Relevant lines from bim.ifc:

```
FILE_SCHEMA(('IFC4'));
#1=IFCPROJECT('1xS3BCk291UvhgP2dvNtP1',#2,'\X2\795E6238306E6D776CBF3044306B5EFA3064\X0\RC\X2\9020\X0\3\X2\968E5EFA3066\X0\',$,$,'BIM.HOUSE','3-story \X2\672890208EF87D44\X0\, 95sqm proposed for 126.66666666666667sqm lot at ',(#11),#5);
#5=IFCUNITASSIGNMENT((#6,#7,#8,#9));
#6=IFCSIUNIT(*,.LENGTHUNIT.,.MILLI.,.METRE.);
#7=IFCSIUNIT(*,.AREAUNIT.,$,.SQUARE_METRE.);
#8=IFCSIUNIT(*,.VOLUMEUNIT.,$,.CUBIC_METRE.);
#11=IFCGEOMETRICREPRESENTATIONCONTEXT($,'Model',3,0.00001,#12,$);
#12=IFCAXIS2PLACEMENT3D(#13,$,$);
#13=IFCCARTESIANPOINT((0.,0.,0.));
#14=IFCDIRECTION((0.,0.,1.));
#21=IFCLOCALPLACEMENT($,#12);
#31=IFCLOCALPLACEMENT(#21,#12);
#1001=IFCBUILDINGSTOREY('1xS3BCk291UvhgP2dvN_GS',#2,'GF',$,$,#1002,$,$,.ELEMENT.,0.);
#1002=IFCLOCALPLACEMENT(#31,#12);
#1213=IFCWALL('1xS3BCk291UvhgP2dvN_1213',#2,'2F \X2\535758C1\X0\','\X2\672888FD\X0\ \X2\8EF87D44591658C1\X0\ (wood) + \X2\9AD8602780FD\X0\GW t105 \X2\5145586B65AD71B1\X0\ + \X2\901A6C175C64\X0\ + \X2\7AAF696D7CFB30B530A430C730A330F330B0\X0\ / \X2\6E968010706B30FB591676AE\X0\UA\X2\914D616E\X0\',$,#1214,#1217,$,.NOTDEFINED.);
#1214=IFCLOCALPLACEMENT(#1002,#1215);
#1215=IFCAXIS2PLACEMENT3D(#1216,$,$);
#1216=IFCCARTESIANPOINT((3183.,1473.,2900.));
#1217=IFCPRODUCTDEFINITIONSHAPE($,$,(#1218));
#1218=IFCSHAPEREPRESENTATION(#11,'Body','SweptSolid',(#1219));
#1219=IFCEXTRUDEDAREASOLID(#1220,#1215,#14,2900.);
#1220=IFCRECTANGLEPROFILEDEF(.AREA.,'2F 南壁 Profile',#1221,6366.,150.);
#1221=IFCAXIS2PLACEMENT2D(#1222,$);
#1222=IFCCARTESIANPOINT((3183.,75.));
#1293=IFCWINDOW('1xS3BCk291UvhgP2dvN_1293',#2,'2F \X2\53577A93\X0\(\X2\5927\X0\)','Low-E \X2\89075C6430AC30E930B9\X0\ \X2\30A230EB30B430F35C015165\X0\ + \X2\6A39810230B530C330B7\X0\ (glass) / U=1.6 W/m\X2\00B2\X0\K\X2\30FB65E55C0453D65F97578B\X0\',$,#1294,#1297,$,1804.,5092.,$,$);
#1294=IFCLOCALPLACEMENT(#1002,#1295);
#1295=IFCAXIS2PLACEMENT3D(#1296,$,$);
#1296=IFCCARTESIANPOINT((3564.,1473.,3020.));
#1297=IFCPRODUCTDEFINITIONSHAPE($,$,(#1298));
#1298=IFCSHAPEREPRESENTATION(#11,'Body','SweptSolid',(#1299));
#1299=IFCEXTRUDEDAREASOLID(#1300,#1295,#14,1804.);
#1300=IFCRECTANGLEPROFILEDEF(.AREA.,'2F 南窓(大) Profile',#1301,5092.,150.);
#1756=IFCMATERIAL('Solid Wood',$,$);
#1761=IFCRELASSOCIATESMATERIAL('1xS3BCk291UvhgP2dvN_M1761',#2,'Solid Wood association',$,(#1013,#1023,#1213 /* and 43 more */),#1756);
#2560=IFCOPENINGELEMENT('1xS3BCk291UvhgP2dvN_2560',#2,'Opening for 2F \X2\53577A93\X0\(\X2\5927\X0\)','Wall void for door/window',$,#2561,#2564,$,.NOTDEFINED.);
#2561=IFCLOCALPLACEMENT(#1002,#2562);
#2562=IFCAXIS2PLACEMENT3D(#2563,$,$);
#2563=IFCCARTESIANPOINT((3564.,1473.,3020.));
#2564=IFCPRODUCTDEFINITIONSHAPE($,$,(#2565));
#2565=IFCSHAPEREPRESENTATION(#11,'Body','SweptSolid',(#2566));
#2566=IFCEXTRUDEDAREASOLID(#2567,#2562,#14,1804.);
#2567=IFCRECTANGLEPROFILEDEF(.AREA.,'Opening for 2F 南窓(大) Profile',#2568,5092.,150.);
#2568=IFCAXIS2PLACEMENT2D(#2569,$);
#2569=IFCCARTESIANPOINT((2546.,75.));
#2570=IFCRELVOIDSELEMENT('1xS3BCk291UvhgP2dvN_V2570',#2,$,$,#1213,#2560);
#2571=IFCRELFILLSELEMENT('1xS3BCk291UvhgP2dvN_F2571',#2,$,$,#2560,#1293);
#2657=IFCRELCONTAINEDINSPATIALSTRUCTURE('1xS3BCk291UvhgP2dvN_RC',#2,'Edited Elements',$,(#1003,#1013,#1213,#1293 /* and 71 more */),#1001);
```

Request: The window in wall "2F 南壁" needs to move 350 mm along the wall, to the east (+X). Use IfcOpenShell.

```python
import ifcopenshell
import ifcopenshell.api.geometry
import ifcopenshell.util.placement

model = ifcopenshell.open("bim.ifc")

window = model.by_guid("1xS3BCk291UvhgP2dvN_1293")
opening = window.FillsVoids[0].RelatingOpeningElement
wall = opening.VoidsElements[0].RelatingBuildingElement

wall_matrix = ifcopenshell.util.placement.get_local_placement(wall.ObjectPlacement)
shift = wall_matrix[:3, 0] * 350.0
before = ifcopenshell.util.placement.get_local_placement(window.ObjectPlacement)[:3, 3].copy()

# The window is not placed relative to its opening, so move both.
for product in (opening, window):
    matrix = ifcopenshell.util.placement.get_local_placement(product.ObjectPlacement)
    matrix[:3, 3] += shift
    ifcopenshell.api.geometry.edit_object_placement(model, product=product, matrix=matrix, is_si=False)

after = ifcopenshell.util.placement.get_local_placement(window.ObjectPlacement)[:3, 3]
print("window moved by", (after - before).round(3) + 0.0)

model.write("bim-out.ifc")
```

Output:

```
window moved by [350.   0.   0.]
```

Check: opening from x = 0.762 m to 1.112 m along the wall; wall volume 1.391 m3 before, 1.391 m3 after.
